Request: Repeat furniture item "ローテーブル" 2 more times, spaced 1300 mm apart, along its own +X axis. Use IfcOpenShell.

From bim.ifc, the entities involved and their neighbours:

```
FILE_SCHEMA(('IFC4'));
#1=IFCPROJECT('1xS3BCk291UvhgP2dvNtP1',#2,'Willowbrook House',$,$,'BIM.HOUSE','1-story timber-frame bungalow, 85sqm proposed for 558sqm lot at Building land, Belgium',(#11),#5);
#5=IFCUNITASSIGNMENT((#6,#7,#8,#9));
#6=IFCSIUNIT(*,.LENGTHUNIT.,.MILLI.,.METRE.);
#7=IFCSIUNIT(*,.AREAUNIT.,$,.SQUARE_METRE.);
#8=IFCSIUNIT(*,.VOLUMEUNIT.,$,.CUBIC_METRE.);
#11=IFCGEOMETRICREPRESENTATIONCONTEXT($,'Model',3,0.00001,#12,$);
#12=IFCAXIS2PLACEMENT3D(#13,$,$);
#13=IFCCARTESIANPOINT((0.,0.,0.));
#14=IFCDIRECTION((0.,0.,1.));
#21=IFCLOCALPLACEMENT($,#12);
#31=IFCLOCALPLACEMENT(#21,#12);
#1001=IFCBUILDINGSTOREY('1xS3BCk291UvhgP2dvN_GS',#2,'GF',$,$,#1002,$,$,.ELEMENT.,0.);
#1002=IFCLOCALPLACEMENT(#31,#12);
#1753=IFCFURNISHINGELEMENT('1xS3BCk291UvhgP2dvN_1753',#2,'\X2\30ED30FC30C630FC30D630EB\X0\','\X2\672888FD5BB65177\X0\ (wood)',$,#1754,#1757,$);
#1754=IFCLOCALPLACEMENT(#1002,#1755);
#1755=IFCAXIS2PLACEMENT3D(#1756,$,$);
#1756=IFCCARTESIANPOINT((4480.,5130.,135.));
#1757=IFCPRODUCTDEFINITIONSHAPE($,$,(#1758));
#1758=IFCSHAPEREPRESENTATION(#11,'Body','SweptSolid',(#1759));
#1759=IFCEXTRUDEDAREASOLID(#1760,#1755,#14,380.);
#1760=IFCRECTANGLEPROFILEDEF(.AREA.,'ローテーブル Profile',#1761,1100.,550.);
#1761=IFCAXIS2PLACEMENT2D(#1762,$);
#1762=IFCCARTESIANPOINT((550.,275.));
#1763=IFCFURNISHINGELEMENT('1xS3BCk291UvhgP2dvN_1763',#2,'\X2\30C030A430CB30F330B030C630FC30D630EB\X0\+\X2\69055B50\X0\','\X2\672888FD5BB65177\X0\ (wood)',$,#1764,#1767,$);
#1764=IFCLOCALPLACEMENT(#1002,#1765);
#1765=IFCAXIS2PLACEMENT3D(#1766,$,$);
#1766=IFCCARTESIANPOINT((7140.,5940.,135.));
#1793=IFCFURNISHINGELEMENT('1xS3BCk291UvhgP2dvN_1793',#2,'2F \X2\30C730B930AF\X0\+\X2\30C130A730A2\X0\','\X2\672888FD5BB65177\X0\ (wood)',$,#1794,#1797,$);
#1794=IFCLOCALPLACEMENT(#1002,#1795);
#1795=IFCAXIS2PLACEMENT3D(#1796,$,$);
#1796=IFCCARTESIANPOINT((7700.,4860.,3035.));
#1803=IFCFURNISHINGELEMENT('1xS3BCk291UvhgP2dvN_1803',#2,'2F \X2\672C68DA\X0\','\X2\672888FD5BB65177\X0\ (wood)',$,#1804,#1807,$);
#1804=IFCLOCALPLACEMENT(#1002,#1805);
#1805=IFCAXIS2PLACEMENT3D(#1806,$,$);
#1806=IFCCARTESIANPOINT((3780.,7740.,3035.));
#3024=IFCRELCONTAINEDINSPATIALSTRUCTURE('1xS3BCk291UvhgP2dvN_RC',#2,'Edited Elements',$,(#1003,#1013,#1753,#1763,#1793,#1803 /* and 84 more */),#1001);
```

```python
import ifcopenshell
import ifcopenshell.api.geometry
import ifcopenshell.api.root
import ifcopenshell.util.element
import ifcopenshell.util.placement
import ifcopenshell.util.unit

model = ifcopenshell.open("bim.ifc")
unit_scale = ifcopenshell.util.unit.calculate_unit_scale(model)


def reuse_history(source, copy):
    """copy_class also copies each property set's owner history, people and application; keep the originals."""
    for rel in copy.IsDefinedBy:
        if rel.is_a("IfcRelDefinesByProperties") and (history := rel.RelatingPropertyDefinition.OwnerHistory):
            rel.RelatingPropertyDefinition.OwnerHistory = source.OwnerHistory
            ifcopenshell.util.element.remove_deep2(model, history)


source = model.by_guid("1xS3BCk291UvhgP2dvN_1753")
base = ifcopenshell.util.placement.get_local_placement(source.ObjectPlacement)
step = base[:3, 0] * 1.3 / unit_scale

for i in range(1, 3):
    copy = ifcopenshell.api.root.copy_class(model, product=source)
    copy.Representation = ifcopenshell.util.element.copy_deep(
        model, source.Representation, exclude=["IfcGeometricRepresentationContext", "IfcRepresentationMap"]
    )
    reuse_history(source, copy)
    matrix = base.copy()
    matrix[:3, 3] += i * step
    print("added at", matrix[:3, 3].round(3) + 0.0)
    ifcopenshell.api.geometry.edit_object_placement(model, product=copy, matrix=matrix, is_si=False)

model.write("bim-out.ifc")
```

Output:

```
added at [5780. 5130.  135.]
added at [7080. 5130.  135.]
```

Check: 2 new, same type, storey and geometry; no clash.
